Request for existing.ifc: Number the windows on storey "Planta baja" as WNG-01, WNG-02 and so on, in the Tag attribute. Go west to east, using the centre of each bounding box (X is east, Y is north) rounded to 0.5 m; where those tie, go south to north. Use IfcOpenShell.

First a look at what the model holds.

```python
import ifcopenshell
import ifcopenshell.util.element
import ifcopenshell.util.placement

model = ifcopenshell.open("existing.ifc")
print(model.schema)
storey = next(s for s in model.by_type("IfcBuildingStorey") if s.Name == "Planta baja")
windows = [e for e in ifcopenshell.util.element.get_decomposition(storey) if e.is_a("IfcWindow")]
for e in sorted(windows, key=lambda e: e.id()):
    origin = ifcopenshell.util.placement.get_local_placement(e.ObjectPlacement)[:3, 3]
    print(e.id(), e.Tag, e.Name, origin.round(2) + 0.0, sep=" | ")
```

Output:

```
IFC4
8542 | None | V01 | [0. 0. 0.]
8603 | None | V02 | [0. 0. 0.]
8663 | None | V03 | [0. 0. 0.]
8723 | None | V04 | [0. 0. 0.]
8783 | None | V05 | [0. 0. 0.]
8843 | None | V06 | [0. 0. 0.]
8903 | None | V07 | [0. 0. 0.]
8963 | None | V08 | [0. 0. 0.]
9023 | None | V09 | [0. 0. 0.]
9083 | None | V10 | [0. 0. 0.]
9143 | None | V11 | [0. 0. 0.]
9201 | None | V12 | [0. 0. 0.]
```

```python
import ifcopenshell
import ifcopenshell.geom
import ifcopenshell.util.element
import ifcopenshell.util.shape

model = ifcopenshell.open("existing.ifc")
settings = ifcopenshell.geom.settings()
settings.set("use-world-coords", True)


def centre(element):
    shape = ifcopenshell.geom.create_shape(settings, element)
    return ifcopenshell.util.shape.get_bbox_centroid(shape.geometry)


storey = next(s for s in model.by_type("IfcBuildingStorey") if s.Name == "Planta baja")
windows = [e for e in ifcopenshell.util.element.get_decomposition(storey) if e.is_a("IfcWindow")]

# Insertion points can sit at a corner or the storey origin, so sort by the geometry (in metres).
centres = {e: centre(e) for e in windows}
windows.sort(key=lambda e: (round(centres[e][0] / 0.5), centres[e][1]))

for i, e in enumerate(windows, start=1):
    number = f"WNG-{i:02d}"
    e.Tag = number
    print(e.id(), number)

model.write("existing_v2.ifc")
```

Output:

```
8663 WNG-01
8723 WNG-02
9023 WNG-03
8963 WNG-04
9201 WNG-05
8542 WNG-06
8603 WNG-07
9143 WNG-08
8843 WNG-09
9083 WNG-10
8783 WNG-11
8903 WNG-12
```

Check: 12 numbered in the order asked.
